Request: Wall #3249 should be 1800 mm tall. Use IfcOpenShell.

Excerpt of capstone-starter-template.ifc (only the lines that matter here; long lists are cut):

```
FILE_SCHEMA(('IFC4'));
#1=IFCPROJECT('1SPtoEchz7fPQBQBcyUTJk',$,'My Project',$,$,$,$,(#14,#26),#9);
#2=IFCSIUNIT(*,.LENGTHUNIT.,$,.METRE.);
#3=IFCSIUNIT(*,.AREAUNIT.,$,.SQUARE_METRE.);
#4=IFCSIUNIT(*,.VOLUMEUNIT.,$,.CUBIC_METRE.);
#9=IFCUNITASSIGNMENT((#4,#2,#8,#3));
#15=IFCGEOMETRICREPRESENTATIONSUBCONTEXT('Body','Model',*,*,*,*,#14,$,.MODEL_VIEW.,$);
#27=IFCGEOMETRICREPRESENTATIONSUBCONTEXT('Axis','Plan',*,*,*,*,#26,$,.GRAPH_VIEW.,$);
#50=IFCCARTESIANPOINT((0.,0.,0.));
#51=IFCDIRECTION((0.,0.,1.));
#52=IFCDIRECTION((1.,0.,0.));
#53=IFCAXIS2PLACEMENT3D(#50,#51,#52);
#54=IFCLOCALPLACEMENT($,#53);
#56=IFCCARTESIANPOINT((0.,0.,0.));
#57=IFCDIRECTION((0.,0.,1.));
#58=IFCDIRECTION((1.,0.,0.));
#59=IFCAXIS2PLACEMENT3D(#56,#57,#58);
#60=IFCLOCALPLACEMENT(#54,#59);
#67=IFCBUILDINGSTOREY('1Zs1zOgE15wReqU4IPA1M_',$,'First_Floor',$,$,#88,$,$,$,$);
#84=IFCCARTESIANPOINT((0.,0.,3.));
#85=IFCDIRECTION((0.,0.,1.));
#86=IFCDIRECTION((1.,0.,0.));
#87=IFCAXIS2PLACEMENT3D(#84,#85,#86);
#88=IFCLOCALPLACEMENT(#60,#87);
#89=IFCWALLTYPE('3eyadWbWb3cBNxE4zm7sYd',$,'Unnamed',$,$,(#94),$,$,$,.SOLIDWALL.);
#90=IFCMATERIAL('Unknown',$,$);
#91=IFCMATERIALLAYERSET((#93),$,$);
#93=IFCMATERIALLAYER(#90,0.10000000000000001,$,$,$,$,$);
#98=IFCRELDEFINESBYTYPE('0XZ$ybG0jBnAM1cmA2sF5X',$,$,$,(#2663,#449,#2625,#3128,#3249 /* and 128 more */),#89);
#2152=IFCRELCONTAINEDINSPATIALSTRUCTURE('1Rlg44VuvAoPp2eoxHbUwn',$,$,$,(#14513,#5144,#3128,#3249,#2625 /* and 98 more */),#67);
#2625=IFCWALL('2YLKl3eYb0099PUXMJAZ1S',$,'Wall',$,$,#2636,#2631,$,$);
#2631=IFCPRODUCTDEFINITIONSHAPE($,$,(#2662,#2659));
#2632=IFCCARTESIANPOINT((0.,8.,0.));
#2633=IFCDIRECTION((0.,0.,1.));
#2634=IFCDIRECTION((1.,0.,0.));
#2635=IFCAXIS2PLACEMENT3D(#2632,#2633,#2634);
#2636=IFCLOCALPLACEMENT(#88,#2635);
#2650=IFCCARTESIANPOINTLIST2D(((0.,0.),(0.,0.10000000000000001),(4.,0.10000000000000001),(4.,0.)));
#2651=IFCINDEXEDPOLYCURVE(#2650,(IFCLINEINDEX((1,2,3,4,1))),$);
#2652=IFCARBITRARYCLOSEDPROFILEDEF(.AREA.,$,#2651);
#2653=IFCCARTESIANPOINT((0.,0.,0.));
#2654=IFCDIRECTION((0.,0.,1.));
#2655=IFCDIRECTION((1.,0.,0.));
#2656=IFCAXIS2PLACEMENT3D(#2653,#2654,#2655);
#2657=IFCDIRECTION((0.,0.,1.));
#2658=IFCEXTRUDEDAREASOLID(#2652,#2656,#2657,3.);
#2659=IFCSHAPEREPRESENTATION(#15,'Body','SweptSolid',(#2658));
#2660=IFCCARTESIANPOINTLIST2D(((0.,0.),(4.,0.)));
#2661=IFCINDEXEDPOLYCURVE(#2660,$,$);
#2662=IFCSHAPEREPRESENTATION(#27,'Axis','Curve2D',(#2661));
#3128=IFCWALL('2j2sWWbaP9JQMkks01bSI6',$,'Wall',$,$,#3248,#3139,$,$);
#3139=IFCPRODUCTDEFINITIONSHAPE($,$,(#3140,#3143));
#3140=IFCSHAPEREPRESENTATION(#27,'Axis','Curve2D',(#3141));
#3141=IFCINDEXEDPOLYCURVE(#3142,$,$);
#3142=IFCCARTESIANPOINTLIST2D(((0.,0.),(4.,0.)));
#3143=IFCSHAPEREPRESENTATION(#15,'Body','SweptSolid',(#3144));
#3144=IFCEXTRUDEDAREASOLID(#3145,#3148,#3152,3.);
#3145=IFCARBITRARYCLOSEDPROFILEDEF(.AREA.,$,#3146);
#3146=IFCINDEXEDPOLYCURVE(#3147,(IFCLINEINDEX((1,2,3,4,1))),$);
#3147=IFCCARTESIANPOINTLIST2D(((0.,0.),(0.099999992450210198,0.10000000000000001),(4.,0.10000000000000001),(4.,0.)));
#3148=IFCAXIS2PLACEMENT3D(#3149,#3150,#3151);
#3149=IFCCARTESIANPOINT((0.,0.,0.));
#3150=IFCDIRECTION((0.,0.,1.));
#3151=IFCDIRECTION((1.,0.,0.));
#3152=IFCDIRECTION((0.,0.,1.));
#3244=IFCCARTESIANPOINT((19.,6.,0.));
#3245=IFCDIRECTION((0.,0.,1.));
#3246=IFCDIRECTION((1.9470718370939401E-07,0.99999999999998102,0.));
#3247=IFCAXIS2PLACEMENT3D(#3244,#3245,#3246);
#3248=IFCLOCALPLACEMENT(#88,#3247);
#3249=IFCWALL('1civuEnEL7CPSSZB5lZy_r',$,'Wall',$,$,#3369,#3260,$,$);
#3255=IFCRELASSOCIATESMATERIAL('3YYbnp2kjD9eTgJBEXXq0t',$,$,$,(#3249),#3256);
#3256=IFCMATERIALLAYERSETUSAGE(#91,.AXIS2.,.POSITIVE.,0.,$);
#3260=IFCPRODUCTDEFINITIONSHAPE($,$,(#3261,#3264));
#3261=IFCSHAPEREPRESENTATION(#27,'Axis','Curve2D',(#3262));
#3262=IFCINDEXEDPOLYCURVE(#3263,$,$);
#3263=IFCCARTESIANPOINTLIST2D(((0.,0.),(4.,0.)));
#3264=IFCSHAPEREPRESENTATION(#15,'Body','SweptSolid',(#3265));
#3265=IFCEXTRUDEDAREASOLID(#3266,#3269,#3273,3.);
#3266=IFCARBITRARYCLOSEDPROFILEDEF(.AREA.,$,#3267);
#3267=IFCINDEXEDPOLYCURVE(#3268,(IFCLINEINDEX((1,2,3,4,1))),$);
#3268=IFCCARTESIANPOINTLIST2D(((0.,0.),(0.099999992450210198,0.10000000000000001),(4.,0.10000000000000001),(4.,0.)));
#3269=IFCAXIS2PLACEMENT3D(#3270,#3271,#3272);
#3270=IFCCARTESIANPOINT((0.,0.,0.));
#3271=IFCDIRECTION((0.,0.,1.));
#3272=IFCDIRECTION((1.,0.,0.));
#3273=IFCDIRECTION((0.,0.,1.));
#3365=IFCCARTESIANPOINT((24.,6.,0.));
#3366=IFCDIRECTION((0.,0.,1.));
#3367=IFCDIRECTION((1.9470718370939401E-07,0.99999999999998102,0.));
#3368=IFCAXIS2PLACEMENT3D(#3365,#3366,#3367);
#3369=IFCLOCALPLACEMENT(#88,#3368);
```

```python
import ifcopenshell
import ifcopenshell.geom
import ifcopenshell.util.representation
import ifcopenshell.util.shape
import ifcopenshell.util.unit

model = ifcopenshell.open("capstone-starter-template.ifc")
unit_scale = ifcopenshell.util.unit.calculate_unit_scale(model)
settings = ifcopenshell.geom.settings()


def volume(element):
    """Net volume in cubic metres, openings subtracted."""
    shape = ifcopenshell.geom.create_shape(settings, element)
    return ifcopenshell.util.shape.get_volume(shape.geometry)


wall = model.by_guid("1civuEnEL7CPSSZB5lZy_r")
before = volume(wall)

body = ifcopenshell.util.representation.get_representation(wall, "Model", "Body")
solid = body.Items[0]
old_height = solid.Depth
solid.Depth = 1.8 / unit_scale
after = volume(wall)

print(f"height {old_height:g} -> {solid.Depth:g}, volume {before:.3f} -> {after:.3f} m3")

model.write("capstone-starter-template_rev.ifc")
```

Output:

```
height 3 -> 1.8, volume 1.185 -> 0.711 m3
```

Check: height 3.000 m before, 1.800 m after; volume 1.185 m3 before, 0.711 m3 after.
